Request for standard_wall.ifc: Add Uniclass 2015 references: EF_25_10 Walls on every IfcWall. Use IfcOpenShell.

First a look at what the model holds.

```python
import ifcopenshell

model = ifcopenshell.open("standard_wall.ifc")
print(model.schema)
print("classifications:", [c.Name for c in model.by_type("IfcClassification")])
for ifc_class in ("IfcDoor", "IfcRoof", "IfcStair", "IfcWall", "IfcWindow"):
    print(ifc_class, len(model.by_type(ifc_class)))
```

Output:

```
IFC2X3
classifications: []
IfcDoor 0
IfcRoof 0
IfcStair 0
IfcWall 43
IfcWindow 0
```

```python
import ifcopenshell
import ifcopenshell.api.classification

model = ifcopenshell.open("standard_wall.ifc")

# IFC2X3 requires Source and Edition and has no link from the project to the system.
system = model.create_entity("IfcClassification", Source="NBS", Edition="2015", Name="Uniclass 2015")

codes = {
    "IfcWall": ("EF_25_10", "Walls"),
}
for ifc_class, (code, name) in codes.items():
    products = model.by_type(ifc_class)
    ifcopenshell.api.classification.add_reference(
        model, products=products, classification=system, identification=code, name=name
    )
    print(code, len(products))

model.write("standard_wall_updated.ifc")
```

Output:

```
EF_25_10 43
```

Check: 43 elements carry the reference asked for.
